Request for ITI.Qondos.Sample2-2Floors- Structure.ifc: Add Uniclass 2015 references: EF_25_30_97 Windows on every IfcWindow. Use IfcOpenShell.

First a look at what the model holds.

```python
import ifcopenshell

model = ifcopenshell.open("ITI.Qondos.Sample2-2Floors- Structure.ifc")
print(model.schema)
print("classifications:", [c.Name for c in model.by_type("IfcClassification")])
for ifc_class in ("IfcDoor", "IfcRoof", "IfcStair", "IfcWall", "IfcWindow"):
    print(ifc_class, len(model.by_type(ifc_class)))
```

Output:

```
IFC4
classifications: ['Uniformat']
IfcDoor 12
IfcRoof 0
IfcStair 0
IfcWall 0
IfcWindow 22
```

```python
import ifcopenshell
import ifcopenshell.api.classification

model = ifcopenshell.open("ITI.Qondos.Sample2-2Floors- Structure.ifc")

system = ifcopenshell.api.classification.add_classification(model, classification="Uniclass 2015")

codes = {
    "IfcWindow": ("EF_25_30_97", "Windows"),
}
for ifc_class, (code, name) in codes.items():
    products = model.by_type(ifc_class)
    ifcopenshell.api.classification.add_reference(
        model, products=products, classification=system, identification=code, name=name
    )
    print(code, len(products))

model.write("ITI.Qondos.Sample2-2Floors- Structure_updated.ifc")
```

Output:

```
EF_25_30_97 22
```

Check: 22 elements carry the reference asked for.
